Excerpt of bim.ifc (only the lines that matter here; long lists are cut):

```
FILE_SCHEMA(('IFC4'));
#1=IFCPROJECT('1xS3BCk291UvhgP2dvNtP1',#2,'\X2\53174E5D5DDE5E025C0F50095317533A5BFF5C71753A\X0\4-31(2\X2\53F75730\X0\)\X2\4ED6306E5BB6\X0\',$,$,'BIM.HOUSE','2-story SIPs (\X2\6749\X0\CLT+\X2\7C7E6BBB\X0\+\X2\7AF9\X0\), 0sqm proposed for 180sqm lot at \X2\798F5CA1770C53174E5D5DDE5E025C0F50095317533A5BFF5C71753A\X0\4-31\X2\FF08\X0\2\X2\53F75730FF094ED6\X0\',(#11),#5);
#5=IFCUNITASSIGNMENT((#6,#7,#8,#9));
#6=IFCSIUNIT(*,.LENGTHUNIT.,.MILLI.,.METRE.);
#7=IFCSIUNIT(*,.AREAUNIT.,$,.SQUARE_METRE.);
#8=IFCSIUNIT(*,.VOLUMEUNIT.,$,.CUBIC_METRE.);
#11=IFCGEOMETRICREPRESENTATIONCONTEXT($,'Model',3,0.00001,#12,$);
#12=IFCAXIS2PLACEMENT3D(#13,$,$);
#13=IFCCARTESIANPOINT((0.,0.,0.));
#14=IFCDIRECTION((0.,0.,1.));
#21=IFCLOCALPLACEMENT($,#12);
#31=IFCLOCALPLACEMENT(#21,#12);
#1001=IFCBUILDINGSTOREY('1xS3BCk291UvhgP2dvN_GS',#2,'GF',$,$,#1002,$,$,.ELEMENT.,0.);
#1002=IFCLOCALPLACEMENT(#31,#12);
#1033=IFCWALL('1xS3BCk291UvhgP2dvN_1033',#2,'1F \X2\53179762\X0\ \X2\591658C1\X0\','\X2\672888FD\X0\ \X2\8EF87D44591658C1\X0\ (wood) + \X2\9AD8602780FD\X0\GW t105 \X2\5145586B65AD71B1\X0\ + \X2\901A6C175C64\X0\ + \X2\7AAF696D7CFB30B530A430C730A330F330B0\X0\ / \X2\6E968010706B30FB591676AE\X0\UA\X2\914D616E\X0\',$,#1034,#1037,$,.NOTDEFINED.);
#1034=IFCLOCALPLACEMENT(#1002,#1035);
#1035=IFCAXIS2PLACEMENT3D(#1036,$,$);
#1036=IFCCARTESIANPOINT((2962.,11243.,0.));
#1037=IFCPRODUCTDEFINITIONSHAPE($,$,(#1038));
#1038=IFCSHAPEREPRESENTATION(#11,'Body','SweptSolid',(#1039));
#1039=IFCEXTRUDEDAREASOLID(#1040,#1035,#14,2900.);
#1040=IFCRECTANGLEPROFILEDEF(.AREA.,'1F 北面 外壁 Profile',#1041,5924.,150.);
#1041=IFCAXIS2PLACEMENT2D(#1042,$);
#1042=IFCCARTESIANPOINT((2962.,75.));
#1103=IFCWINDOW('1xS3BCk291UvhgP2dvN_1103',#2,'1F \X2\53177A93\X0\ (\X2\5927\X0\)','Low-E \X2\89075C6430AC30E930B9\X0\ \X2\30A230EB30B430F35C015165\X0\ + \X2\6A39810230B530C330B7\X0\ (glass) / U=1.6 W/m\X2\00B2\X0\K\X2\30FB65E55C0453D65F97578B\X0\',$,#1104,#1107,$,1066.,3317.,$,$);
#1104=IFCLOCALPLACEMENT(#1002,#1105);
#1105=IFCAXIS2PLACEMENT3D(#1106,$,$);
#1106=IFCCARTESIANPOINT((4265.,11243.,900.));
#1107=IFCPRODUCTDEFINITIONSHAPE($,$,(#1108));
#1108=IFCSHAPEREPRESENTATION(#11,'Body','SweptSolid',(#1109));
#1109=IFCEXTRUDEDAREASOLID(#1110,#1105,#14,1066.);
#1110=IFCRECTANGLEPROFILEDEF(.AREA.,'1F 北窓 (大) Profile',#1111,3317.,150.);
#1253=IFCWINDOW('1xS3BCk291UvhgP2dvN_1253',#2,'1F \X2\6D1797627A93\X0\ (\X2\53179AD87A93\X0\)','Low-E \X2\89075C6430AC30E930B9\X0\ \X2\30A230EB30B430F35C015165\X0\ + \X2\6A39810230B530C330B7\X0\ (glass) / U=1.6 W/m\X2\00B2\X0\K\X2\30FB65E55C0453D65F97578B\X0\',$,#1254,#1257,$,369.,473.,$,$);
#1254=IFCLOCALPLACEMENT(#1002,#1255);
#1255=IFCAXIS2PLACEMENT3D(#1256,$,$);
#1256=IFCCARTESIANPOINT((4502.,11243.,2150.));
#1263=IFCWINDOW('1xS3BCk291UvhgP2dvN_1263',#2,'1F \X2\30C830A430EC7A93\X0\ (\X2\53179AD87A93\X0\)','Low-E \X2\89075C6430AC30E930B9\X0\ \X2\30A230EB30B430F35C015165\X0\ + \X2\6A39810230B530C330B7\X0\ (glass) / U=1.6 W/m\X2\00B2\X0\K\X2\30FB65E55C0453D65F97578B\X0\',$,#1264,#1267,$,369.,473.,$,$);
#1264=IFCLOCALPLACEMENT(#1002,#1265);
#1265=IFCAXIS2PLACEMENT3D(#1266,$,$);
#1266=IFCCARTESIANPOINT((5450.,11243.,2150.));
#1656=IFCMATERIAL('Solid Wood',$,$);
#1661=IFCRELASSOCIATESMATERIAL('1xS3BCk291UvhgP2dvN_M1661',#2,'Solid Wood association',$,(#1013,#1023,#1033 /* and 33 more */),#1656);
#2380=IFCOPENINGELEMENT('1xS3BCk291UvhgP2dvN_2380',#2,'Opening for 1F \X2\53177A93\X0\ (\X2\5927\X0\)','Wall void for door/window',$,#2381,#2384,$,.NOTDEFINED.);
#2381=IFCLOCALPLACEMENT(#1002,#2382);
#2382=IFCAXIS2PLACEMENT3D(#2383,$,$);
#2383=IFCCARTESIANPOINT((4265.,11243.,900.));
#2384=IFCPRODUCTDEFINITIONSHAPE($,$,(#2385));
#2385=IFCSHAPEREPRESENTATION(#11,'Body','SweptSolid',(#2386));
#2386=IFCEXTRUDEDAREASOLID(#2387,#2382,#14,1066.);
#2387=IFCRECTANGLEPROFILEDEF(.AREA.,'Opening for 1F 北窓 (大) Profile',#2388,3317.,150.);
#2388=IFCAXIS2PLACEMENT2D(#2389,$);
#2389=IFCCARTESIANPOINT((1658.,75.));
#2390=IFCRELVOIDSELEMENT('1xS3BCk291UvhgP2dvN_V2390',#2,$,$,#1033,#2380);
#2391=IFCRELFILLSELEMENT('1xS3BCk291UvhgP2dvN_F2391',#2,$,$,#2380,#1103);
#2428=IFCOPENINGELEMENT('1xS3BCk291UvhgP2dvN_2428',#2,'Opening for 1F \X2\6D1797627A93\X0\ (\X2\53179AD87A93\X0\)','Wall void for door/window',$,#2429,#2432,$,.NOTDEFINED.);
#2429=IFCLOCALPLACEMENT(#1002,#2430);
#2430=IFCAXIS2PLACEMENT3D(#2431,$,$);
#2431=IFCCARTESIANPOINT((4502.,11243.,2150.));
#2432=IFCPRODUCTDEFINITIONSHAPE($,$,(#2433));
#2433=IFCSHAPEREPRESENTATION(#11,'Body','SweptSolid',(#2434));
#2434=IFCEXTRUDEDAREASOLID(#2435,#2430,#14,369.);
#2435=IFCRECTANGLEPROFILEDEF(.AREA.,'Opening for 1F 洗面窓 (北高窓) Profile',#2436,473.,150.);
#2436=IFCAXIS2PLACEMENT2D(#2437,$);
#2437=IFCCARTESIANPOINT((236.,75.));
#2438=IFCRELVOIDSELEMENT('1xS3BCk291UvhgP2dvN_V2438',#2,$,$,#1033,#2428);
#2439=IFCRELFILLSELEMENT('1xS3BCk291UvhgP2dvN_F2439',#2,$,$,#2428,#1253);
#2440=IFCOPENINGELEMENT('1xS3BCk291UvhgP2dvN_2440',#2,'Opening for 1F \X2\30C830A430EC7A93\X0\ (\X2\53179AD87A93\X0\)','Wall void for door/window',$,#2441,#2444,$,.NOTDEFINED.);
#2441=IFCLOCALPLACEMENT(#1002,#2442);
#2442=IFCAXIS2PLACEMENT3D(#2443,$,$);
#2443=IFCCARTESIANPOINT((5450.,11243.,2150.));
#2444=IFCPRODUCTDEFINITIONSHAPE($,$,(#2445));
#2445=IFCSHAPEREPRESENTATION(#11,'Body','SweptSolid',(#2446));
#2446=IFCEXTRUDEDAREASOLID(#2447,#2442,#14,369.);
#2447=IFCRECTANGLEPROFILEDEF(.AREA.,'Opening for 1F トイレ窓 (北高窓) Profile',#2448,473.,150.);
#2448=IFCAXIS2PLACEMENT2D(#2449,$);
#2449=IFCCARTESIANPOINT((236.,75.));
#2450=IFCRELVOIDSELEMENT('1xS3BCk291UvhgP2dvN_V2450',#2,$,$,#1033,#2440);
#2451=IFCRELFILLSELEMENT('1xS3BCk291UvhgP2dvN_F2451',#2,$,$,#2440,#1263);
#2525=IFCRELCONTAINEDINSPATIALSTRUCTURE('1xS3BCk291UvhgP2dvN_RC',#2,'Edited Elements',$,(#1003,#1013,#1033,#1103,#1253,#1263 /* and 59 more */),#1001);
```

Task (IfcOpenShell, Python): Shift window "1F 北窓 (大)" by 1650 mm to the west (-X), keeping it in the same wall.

```python
import ifcopenshell
import ifcopenshell.api.geometry
import ifcopenshell.util.placement
import ifcopenshell.util.unit

model = ifcopenshell.open("bim.ifc")
unit_scale = ifcopenshell.util.unit.calculate_unit_scale(model)

window = model.by_guid("1xS3BCk291UvhgP2dvN_1103")
opening = window.FillsVoids[0].RelatingOpeningElement
wall = opening.VoidsElements[0].RelatingBuildingElement

wall_matrix = ifcopenshell.util.placement.get_local_placement(wall.ObjectPlacement)
shift = wall_matrix[:3, 0] * -1.65 / unit_scale
before = ifcopenshell.util.placement.get_local_placement(window.ObjectPlacement)[:3, 3].copy()

# The window is not placed relative to its opening, so move both.
for product in (opening, window):
    matrix = ifcopenshell.util.placement.get_local_placement(product.ObjectPlacement)
    matrix[:3, 3] += shift
    ifcopenshell.api.geometry.edit_object_placement(model, product=product, matrix=matrix, is_si=False)

after = ifcopenshell.util.placement.get_local_placement(window.ObjectPlacement)[:3, 3]
print("window moved by", (after - before).round(3) + 0.0)

model.write("bim_updated.ifc")
```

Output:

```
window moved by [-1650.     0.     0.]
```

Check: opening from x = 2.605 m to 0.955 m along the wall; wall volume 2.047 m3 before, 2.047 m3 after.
